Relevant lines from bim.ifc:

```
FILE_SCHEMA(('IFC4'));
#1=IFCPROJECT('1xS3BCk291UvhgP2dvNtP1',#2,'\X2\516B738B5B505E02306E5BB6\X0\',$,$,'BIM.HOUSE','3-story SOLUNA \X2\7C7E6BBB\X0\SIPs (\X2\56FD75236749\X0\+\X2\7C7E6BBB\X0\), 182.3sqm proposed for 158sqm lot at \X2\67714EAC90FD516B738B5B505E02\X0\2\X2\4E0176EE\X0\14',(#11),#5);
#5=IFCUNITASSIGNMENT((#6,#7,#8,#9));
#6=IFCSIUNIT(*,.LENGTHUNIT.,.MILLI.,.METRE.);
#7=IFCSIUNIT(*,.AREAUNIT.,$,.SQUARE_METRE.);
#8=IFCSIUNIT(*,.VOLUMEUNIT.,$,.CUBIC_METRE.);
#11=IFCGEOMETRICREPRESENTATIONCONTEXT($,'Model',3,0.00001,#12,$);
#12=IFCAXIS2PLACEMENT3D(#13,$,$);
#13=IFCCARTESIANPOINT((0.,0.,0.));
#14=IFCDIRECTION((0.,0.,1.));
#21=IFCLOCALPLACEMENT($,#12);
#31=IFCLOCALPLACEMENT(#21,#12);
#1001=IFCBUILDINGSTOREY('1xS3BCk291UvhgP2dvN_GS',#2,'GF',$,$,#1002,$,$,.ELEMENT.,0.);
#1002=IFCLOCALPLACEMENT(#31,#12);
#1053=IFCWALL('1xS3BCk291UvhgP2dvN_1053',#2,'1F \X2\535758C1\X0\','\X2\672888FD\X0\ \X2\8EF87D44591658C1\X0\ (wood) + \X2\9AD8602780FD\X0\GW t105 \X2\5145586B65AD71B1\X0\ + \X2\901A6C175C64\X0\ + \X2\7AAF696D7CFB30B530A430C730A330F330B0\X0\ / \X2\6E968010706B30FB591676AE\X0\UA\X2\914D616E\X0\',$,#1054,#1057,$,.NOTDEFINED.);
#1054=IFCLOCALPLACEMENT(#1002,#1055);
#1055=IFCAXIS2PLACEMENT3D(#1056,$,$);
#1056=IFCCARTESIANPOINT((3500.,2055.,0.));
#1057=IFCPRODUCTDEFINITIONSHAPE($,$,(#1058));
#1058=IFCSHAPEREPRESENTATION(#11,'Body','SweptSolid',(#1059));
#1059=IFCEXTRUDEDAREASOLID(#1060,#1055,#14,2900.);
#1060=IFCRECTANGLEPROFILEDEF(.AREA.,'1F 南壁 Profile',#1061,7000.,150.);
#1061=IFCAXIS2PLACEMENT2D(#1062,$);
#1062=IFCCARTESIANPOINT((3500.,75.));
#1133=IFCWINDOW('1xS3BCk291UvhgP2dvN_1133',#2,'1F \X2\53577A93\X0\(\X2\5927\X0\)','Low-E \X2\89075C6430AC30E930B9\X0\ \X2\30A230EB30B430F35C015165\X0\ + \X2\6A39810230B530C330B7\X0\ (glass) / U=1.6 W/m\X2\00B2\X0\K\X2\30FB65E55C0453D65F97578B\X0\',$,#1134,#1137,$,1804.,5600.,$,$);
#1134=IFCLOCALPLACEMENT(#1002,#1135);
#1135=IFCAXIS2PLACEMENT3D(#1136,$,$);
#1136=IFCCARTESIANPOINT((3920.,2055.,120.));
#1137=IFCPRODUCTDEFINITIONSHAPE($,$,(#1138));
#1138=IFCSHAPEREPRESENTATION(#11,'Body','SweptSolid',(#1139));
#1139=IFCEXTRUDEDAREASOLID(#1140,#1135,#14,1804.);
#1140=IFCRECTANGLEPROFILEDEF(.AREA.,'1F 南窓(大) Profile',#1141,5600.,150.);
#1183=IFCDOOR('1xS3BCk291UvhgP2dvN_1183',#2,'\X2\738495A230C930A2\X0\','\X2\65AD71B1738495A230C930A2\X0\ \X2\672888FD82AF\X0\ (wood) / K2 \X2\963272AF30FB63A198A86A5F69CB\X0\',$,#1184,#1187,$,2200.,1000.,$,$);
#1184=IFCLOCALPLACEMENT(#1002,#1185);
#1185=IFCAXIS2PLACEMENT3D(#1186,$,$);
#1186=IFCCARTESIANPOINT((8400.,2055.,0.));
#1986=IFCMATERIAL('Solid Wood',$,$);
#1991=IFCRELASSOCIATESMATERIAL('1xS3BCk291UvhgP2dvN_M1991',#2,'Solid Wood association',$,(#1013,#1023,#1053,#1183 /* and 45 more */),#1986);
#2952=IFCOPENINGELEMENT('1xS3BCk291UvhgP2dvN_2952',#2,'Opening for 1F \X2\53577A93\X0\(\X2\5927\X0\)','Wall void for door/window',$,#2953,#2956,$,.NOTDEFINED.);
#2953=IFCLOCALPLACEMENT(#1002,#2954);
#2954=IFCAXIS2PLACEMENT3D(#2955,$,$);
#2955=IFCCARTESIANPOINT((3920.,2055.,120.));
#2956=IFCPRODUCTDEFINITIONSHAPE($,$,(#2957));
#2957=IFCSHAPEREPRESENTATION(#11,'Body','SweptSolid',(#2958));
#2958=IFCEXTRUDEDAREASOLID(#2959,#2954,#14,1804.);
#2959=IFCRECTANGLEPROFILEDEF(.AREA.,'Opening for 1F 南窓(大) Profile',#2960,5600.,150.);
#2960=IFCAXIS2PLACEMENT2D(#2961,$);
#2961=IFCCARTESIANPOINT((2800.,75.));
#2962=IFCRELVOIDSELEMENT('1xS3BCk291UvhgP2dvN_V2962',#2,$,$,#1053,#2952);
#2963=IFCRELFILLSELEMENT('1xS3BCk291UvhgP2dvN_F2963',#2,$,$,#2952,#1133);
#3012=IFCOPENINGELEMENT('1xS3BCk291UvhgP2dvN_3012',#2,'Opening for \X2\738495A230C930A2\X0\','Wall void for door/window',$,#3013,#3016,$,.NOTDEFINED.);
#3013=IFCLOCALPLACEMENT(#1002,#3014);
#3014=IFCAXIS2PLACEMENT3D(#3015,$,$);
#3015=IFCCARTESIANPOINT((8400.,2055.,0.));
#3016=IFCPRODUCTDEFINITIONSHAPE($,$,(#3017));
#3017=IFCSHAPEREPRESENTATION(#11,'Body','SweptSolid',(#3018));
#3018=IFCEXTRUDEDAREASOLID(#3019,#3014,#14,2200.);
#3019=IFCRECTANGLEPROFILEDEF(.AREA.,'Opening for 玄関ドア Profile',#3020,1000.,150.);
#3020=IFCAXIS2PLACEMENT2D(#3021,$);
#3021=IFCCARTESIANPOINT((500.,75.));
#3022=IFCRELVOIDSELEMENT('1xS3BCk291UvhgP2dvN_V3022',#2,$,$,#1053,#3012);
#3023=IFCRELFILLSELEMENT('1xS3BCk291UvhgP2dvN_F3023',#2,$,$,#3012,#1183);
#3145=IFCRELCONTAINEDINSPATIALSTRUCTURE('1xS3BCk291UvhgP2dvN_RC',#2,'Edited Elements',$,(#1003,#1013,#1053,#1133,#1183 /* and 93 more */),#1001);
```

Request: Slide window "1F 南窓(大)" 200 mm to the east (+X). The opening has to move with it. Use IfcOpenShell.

```python
import ifcopenshell
import ifcopenshell.api.geometry
import ifcopenshell.util.placement
import ifcopenshell.util.unit

model = ifcopenshell.open("bim.ifc")
unit_scale = ifcopenshell.util.unit.calculate_unit_scale(model)

window = model.by_id(1133)
opening = window.FillsVoids[0].RelatingOpeningElement
wall = opening.VoidsElements[0].RelatingBuildingElement

wall_matrix = ifcopenshell.util.placement.get_local_placement(wall.ObjectPlacement)
shift = wall_matrix[:3, 0] * 0.2 / unit_scale
before = ifcopenshell.util.placement.get_local_placement(window.ObjectPlacement)[:3, 3].copy()

# The window is not placed relative to its opening, so move both.
for product in (opening, window):
    matrix = ifcopenshell.util.placement.get_local_placement(product.ObjectPlacement)
    matrix[:3, 3] += shift
    ifcopenshell.api.geometry.edit_object_placement(model, product=product, matrix=matrix, is_si=False)

after = ifcopenshell.util.placement.get_local_placement(window.ObjectPlacement)[:3, 3]
print("window moved by", (after - before).round(3) + 0.0)

model.write("bim_v2.ifc")
```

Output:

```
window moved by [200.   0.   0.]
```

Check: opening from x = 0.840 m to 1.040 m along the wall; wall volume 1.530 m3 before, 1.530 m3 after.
